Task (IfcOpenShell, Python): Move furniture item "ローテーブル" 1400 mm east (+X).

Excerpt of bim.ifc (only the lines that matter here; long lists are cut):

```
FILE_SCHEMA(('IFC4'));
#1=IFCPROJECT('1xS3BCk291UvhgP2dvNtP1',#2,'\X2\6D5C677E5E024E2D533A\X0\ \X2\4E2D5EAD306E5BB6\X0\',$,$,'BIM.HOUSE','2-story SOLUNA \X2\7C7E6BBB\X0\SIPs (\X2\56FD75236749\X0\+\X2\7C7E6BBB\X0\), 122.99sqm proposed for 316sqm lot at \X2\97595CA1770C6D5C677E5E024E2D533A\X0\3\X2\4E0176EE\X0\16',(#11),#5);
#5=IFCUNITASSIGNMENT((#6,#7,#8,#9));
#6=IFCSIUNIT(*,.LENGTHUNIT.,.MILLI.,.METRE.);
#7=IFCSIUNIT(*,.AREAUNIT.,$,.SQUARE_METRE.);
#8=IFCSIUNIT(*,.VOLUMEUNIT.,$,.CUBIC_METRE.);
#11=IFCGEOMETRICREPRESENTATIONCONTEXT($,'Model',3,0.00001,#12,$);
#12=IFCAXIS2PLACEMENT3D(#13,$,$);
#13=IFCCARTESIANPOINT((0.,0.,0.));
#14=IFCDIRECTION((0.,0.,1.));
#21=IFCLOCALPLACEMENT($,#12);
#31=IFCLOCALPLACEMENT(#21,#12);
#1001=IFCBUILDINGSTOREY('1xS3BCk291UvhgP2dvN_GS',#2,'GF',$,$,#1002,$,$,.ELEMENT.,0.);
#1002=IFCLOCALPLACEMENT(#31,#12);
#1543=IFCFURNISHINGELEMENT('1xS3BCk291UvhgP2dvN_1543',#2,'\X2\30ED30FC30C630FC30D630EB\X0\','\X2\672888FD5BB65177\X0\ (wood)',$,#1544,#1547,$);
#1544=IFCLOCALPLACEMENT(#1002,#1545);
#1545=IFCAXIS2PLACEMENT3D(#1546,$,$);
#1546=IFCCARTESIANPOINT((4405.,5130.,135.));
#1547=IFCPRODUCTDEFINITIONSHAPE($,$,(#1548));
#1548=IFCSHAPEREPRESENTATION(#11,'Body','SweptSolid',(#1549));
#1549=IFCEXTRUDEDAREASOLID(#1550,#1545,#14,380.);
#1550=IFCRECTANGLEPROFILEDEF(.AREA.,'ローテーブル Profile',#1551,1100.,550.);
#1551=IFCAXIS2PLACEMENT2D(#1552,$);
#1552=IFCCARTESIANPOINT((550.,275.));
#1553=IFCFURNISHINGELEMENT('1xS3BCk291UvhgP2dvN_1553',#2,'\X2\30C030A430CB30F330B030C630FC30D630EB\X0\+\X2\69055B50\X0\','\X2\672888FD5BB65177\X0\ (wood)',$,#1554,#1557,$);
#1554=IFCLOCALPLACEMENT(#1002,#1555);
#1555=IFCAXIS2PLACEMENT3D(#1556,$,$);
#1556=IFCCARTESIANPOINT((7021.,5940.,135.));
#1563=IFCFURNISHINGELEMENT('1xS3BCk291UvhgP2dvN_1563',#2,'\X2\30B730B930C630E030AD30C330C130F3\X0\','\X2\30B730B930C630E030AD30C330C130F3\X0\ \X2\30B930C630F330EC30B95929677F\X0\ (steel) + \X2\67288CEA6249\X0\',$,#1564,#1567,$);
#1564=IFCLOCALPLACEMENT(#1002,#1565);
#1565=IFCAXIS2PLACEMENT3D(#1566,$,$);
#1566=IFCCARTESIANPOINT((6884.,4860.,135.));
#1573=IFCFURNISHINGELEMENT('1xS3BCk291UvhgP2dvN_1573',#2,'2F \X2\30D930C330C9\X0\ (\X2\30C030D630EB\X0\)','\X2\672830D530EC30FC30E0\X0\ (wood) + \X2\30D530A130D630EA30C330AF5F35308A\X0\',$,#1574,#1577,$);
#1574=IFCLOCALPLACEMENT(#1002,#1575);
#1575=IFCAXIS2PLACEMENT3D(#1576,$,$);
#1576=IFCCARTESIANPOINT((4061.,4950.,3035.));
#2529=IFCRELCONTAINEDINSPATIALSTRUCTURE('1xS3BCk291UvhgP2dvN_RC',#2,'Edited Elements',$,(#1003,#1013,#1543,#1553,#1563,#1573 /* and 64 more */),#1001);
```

```python
import ifcopenshell
import ifcopenshell.api.geometry
import ifcopenshell.util.placement
import ifcopenshell.util.unit

model = ifcopenshell.open("bim.ifc")
unit_scale = ifcopenshell.util.unit.calculate_unit_scale(model)

item = model.by_guid("1xS3BCk291UvhgP2dvN_1543")
matrix = ifcopenshell.util.placement.get_local_placement(item.ObjectPlacement)
matrix[0, 3] += 1.4 / unit_scale
ifcopenshell.api.geometry.edit_object_placement(model, product=item, matrix=matrix, is_si=False)

print(ifcopenshell.util.placement.get_local_placement(item.ObjectPlacement).round(3) + 0.0)

model.write("bim_v2.ifc")
```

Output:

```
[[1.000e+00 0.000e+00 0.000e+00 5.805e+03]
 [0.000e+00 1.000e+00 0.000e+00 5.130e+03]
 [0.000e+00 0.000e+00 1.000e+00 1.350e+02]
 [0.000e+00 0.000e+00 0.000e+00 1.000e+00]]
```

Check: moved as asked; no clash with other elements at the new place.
